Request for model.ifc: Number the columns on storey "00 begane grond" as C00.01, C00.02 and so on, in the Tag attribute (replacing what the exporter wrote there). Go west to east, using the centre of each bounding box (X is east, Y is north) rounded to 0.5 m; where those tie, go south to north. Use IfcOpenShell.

First a look at what the model holds.

```python
import ifcopenshell
import ifcopenshell.util.element
import ifcopenshell.util.placement

model = ifcopenshell.open("model.ifc")
print(model.schema)
storey = next(s for s in model.by_type("IfcBuildingStorey") if s.Name == "00 begane grond")
columns = [e for e in ifcopenshell.util.element.get_decomposition(storey) if e.is_a("IfcColumn")]
for e in sorted(columns, key=lambda e: e.id()):
    origin = ifcopenshell.util.placement.get_local_placement(e.ObjectPlacement)[:3, 3]
    print(e.id(), e.Tag, e.Name, origin.round(2) + 0.0, sep=" | ")
```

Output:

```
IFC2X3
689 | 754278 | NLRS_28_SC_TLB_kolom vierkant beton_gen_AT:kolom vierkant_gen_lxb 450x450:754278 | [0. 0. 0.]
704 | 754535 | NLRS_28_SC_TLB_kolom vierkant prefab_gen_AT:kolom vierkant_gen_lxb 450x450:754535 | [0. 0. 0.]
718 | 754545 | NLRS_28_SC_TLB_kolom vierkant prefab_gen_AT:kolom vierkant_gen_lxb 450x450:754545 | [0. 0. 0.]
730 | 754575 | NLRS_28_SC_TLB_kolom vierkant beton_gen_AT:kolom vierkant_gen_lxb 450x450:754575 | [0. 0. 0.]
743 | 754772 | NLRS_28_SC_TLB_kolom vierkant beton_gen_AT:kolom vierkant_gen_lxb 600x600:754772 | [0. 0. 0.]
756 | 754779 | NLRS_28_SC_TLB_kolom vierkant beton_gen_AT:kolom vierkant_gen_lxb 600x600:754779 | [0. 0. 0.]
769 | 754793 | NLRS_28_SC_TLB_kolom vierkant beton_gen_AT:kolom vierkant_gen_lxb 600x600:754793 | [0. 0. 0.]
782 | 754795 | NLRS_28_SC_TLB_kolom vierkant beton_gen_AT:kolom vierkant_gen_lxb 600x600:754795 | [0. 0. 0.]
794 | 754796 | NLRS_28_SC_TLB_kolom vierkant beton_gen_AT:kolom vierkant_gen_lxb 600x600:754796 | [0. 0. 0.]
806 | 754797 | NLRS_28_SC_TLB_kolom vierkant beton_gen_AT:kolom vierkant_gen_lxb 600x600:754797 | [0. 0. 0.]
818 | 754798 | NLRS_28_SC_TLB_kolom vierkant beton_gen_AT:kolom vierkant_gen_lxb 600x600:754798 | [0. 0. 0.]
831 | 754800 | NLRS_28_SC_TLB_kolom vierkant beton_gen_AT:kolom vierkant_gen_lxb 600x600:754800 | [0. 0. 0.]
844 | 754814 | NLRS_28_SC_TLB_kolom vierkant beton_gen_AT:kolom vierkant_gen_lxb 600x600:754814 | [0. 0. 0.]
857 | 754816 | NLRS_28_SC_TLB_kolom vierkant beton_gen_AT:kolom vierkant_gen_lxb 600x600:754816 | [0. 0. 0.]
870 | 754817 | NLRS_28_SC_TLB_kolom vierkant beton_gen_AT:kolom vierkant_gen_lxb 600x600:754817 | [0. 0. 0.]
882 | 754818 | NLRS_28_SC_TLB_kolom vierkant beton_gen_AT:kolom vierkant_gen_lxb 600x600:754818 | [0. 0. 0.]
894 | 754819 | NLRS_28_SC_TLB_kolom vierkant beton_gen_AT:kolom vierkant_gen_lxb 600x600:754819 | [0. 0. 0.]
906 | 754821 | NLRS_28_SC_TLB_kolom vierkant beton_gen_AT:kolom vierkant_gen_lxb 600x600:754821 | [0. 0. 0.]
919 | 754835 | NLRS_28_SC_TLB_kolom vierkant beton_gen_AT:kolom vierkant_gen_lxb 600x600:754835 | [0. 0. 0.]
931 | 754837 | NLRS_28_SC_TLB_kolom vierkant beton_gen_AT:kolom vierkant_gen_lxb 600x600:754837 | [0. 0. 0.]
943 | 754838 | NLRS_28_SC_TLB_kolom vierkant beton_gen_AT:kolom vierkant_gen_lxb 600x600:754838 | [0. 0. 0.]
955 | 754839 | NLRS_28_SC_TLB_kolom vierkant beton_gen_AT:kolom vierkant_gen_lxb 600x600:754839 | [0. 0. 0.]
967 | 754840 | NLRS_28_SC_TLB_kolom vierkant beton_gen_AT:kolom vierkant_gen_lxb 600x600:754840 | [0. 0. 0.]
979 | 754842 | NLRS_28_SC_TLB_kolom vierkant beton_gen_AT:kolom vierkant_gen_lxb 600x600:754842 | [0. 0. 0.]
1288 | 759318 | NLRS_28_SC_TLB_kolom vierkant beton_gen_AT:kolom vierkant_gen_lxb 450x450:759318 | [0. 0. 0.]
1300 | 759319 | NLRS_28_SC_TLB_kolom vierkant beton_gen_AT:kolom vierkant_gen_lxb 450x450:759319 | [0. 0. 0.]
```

```python
import ifcopenshell
import ifcopenshell.geom
import ifcopenshell.util.element
import ifcopenshell.util.shape

model = ifcopenshell.open("model.ifc")
settings = ifcopenshell.geom.settings()
settings.set("use-world-coords", True)


def centre(element):
    shape = ifcopenshell.geom.create_shape(settings, element)
    return ifcopenshell.util.shape.get_bbox_centroid(shape.geometry)


storey = next(s for s in model.by_type("IfcBuildingStorey") if s.Name == "00 begane grond")
columns = [e for e in ifcopenshell.util.element.get_decomposition(storey) if e.is_a("IfcColumn")]

# Insertion points can sit at a corner or the storey origin, so sort by the geometry (in metres).
centres = {e: centre(e) for e in columns}
columns.sort(key=lambda e: (round(centres[e][0] / 0.5), centres[e][1]))

for i, e in enumerate(columns, start=1):
    number = f"C00.{i:02d}"
    e.Tag = number
    print(e.id(), number)

model.write("model-out.ifc")
```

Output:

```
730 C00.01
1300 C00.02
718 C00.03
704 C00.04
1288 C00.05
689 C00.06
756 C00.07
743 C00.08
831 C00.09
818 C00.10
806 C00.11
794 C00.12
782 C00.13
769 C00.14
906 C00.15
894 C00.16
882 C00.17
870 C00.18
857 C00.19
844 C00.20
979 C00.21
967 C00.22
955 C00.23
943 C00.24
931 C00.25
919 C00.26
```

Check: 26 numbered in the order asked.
